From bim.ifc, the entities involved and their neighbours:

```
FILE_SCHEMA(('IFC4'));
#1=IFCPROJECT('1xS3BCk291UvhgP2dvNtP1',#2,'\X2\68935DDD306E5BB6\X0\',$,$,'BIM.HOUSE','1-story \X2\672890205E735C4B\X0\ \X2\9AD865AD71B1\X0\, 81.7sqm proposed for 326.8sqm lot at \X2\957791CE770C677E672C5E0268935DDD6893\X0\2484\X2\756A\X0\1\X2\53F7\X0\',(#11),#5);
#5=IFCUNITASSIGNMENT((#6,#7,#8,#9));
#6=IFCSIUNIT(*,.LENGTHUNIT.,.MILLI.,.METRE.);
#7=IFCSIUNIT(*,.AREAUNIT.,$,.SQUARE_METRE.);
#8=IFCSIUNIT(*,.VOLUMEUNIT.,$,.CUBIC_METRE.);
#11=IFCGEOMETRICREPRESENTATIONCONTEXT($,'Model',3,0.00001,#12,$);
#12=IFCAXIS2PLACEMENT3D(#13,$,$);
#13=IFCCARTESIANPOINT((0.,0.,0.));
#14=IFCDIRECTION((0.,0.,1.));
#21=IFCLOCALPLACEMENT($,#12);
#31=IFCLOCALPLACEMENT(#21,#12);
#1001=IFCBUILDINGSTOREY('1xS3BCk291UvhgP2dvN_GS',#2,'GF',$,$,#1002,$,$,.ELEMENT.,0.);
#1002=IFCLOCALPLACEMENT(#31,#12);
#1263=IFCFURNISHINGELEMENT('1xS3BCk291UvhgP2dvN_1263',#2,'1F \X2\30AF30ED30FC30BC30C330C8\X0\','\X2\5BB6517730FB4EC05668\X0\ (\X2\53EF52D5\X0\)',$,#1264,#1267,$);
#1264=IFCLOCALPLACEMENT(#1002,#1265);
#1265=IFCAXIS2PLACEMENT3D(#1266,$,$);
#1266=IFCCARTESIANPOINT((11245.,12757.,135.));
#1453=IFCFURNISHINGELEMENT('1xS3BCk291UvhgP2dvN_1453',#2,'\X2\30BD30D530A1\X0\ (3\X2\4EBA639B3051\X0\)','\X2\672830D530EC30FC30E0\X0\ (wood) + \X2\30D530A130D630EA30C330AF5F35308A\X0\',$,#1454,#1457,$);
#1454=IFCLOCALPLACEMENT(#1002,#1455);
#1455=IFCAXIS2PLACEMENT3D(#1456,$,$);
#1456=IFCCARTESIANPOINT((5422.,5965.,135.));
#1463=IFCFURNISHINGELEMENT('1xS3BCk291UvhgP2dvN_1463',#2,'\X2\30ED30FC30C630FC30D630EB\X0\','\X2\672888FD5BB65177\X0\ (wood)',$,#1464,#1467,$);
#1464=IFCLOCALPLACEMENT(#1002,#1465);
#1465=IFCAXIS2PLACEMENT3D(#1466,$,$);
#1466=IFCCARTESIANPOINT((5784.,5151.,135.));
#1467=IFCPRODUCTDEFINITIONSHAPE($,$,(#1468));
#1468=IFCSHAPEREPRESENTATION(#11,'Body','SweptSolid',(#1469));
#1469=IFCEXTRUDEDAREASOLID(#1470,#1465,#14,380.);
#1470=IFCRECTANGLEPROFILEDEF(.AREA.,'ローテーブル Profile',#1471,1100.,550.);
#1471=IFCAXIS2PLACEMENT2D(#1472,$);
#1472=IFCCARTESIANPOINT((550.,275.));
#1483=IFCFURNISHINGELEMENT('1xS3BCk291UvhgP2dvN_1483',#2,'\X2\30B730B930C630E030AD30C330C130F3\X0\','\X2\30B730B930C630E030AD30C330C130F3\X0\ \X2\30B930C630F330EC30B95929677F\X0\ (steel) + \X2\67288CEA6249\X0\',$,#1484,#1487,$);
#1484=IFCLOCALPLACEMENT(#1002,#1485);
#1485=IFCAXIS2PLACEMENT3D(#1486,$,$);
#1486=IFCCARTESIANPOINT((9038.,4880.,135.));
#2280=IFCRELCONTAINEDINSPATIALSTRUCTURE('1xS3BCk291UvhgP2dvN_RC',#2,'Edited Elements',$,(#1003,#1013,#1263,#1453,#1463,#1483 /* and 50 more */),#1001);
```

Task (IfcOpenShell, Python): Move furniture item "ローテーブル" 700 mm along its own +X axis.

```python
import ifcopenshell
import ifcopenshell.api.geometry
import ifcopenshell.util.placement

model = ifcopenshell.open("bim.ifc")

item = model.by_id(1463)
matrix = ifcopenshell.util.placement.get_local_placement(item.ObjectPlacement)
matrix[:3, 3] += matrix[:3, 0] * 700.0
ifcopenshell.api.geometry.edit_object_placement(model, product=item, matrix=matrix, is_si=False)

print(ifcopenshell.util.placement.get_local_placement(item.ObjectPlacement).round(3) + 0.0)

model.write("bim-out.ifc")
```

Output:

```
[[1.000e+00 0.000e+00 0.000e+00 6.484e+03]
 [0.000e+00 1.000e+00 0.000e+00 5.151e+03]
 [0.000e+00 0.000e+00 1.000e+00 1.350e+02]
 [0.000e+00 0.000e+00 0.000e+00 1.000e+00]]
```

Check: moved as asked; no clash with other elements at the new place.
